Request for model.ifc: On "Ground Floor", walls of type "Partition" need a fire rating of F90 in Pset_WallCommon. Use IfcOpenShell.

First a look at what the model holds.

```python
import ifcopenshell
import ifcopenshell.util.element

model = ifcopenshell.open("model.ifc")
print(model.schema)
storey = next(s for s in model.by_type("IfcBuildingStorey") if s.Name == "Ground Floor")
walls = [e for e in ifcopenshell.util.element.get_decomposition(storey) if e.is_a("IfcWall")]
seen = {}
for e in walls:
    element_type = ifcopenshell.util.element.get_type(e)
    key = (element_type.Name if element_type != e and element_type else None, ifcopenshell.util.element.get_pset(e, "Pset_WallCommon", "FireRating"))
    seen[key] = seen.get(key, 0) + 1
for (name, value), count in sorted(seen.items(), key=str):
    print(count, "x", name, "|", value)
```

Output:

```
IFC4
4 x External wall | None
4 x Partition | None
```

```python
import ifcopenshell
import ifcopenshell.api.pset
import ifcopenshell.util.element

model = ifcopenshell.open("model.ifc")

storey = next(s for s in model.by_type("IfcBuildingStorey") if s.Name == "Ground Floor")
walls = [e for e in ifcopenshell.util.element.get_decomposition(storey) if e.is_a("IfcWall")]

count = 0
for e in walls:
    element_type = ifcopenshell.util.element.get_type(e)
    if element_type in (None, e) or element_type.Name != "Partition":
        continue
    # add_pset returns the element's existing set when there is one.
    pset = ifcopenshell.api.pset.add_pset(model, product=e, name="Pset_WallCommon")
    ifcopenshell.api.pset.edit_pset(model, pset=pset, properties={"FireRating": "F90"})
    count += 1

print(count, "walls updated")

model.write("model_v2.ifc")
```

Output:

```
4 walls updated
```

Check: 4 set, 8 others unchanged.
